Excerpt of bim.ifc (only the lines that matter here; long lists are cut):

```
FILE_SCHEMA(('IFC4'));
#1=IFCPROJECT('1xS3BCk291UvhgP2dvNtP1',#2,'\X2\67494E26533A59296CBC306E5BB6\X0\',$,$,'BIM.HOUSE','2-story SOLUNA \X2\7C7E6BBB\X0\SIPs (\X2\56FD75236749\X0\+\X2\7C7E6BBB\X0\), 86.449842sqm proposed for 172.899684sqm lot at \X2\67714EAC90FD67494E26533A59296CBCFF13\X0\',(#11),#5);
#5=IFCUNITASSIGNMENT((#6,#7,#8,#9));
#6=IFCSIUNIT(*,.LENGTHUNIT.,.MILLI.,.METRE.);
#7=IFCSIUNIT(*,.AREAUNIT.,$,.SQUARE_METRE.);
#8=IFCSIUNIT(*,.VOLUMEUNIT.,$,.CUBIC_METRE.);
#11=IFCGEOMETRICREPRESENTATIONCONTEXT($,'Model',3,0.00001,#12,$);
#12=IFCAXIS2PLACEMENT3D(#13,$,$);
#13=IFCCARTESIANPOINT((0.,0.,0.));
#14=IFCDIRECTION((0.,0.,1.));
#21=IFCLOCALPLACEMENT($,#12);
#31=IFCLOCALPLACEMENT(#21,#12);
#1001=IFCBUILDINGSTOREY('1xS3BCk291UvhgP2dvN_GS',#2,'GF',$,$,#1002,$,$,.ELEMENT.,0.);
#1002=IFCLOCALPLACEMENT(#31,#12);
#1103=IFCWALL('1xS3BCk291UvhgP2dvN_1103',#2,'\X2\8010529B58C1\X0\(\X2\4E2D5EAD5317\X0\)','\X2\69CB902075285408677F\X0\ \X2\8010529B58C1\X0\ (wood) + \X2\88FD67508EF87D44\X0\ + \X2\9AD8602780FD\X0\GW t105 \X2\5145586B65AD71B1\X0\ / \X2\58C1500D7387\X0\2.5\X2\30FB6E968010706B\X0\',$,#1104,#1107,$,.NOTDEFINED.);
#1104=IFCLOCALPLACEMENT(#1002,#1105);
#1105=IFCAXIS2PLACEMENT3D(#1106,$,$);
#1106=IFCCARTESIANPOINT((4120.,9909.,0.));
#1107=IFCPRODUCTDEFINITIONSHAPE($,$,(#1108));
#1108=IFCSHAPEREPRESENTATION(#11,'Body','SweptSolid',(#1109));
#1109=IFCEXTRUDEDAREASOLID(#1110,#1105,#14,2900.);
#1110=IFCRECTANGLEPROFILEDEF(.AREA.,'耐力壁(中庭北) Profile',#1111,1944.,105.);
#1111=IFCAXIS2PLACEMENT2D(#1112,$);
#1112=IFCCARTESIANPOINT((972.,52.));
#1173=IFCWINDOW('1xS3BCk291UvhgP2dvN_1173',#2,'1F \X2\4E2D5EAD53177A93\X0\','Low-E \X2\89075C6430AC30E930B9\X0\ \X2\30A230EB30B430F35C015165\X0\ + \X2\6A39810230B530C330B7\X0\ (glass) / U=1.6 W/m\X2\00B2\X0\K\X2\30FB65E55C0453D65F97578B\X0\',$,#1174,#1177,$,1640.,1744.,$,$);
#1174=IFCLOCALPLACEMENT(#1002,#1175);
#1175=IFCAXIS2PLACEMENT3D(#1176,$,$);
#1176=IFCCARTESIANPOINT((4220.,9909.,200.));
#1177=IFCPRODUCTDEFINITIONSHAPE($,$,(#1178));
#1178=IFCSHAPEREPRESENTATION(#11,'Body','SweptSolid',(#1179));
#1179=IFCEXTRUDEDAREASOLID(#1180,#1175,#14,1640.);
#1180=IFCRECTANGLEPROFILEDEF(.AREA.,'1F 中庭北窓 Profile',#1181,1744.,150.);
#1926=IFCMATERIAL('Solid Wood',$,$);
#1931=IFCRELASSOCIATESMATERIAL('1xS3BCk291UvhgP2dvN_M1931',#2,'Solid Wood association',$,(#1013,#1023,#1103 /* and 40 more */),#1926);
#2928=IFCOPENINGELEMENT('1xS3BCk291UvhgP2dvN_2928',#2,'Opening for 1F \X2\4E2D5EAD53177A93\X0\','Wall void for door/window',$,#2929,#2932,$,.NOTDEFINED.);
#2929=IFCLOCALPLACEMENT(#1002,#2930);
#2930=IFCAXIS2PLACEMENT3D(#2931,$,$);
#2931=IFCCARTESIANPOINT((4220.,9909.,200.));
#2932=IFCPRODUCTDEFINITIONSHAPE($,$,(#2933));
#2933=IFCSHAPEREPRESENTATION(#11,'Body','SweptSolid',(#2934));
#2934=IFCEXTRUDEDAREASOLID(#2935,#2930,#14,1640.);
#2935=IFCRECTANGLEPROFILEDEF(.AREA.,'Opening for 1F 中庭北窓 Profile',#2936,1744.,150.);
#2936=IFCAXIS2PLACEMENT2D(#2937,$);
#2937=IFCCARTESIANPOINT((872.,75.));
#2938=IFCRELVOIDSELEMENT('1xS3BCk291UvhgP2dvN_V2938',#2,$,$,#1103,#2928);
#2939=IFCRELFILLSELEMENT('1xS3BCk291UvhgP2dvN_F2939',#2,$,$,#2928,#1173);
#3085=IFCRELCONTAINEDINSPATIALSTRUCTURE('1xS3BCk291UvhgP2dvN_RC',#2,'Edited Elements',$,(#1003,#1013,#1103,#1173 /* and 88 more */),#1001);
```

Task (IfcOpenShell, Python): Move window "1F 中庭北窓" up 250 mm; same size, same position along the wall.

```python
import numpy as np
import ifcopenshell
import ifcopenshell.api.geometry
import ifcopenshell.util.placement
import ifcopenshell.util.unit

model = ifcopenshell.open("bim.ifc")
unit_scale = ifcopenshell.util.unit.calculate_unit_scale(model)

window = model.by_id(1173)
opening = window.FillsVoids[0].RelatingOpeningElement
dz = 250.0

shift = np.array([0.0, 0.0, dz])
# The window is not placed relative to its opening, so move both.
for product in (opening, window):
    matrix = ifcopenshell.util.placement.get_local_placement(product.ObjectPlacement)
    matrix[:3, 3] += shift
    ifcopenshell.api.geometry.edit_object_placement(model, product=product, matrix=matrix, is_si=False)

print(f"moved by {dz * unit_scale:+.3f} m")

model.write("bim_edited.ifc")
```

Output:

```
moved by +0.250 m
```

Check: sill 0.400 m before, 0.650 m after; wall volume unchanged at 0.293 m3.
